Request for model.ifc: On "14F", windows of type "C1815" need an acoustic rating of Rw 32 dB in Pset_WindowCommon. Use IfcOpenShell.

First a look at what the model holds.

```python
import ifcopenshell
import ifcopenshell.util.element

model = ifcopenshell.open("model.ifc")
print(model.schema)
storey = next(s for s in model.by_type("IfcBuildingStorey") if s.Name == "14F")
windows = [e for e in ifcopenshell.util.element.get_decomposition(storey) if e.is_a("IfcWindow")]
seen = {}
for e in windows:
    element_type = ifcopenshell.util.element.get_type(e)
    key = (element_type.Name if element_type != e and element_type else None, ifcopenshell.util.element.get_pset(e, "Pset_WindowCommon", "AcousticRating"))
    seen[key] = seen.get(key, 0) + 1
for (name, value), count in sorted(seen.items(), key=str):
    print(count, "x", name, "|", value)
```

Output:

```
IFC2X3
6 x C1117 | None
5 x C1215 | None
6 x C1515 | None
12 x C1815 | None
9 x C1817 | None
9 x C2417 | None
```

```python
import ifcopenshell
import ifcopenshell.api.pset
import ifcopenshell.util.element

model = ifcopenshell.open("model.ifc")

storey = next(s for s in model.by_type("IfcBuildingStorey") if s.Name == "14F")
windows = [e for e in ifcopenshell.util.element.get_decomposition(storey) if e.is_a("IfcWindow")]

count = 0
for e in windows:
    element_type = ifcopenshell.util.element.get_type(e)
    if element_type in (None, e) or element_type.Name != "C1815":
        continue
    # add_pset returns the element's existing set when there is one.
    pset = ifcopenshell.api.pset.add_pset(model, product=e, name="Pset_WindowCommon")
    ifcopenshell.api.pset.edit_pset(model, pset=pset, properties={"AcousticRating": "Rw 32 dB"})
    count += 1

print(count, "windows updated")

model.write("model_edited.ifc")
```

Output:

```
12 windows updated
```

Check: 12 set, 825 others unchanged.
